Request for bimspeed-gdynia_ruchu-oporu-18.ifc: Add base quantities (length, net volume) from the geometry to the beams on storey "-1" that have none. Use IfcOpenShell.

First a look at what the model holds.

```python
import ifcopenshell
import ifcopenshell.util.element
import ifcopenshell.util.unit

model = ifcopenshell.open("bimspeed-gdynia_ruchu-oporu-18.ifc")
print(model.schema)
for unit_type in ("LENGTHUNIT", "AREAUNIT", "VOLUMEUNIT"):
    print(unit_type, ifcopenshell.util.unit.calculate_unit_scale(model, unit_type))
storey = next(s for s in model.by_type("IfcBuildingStorey") if s.Name == "-1")
beams = [e for e in ifcopenshell.util.element.get_decomposition(storey) if e.is_a("IfcBeam")]
for e in sorted(beams, key=lambda e: e.id()):
    print(e.id(), e.is_a(), e.Name, list(ifcopenshell.util.element.get_psets(e, qtos_only=True)), sep=" | ")
```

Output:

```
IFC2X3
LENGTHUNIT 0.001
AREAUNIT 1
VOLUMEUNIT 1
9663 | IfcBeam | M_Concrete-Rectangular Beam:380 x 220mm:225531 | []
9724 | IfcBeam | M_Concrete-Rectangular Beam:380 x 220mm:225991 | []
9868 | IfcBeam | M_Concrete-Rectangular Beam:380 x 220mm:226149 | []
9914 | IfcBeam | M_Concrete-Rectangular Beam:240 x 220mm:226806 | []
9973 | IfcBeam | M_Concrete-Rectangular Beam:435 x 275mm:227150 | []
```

```python
import ifcopenshell
import ifcopenshell.api.pset
import ifcopenshell.geom
import ifcopenshell.util.element
import ifcopenshell.util.shape
import ifcopenshell.util.unit

model = ifcopenshell.open("bimspeed-gdynia_ruchu-oporu-18.ifc")
unit_scale = ifcopenshell.util.unit.calculate_unit_scale(model)
volume_scale = ifcopenshell.util.unit.calculate_unit_scale(model, "VOLUMEUNIT")
settings = ifcopenshell.geom.settings()

storey = next(s for s in model.by_type("IfcBuildingStorey") if s.Name == "-1")
beams = [e for e in ifcopenshell.util.element.get_decomposition(storey) if e.is_a("IfcBeam")]

for e in sorted(beams, key=lambda e: e.id()):
    if ifcopenshell.util.element.get_psets(e, qtos_only=True, should_inherit=False):
        continue
    # Geometry comes back in metres, in the element's own axes.
    shape = ifcopenshell.geom.create_shape(settings, e)
    values = {
        "Length": ifcopenshell.util.shape.get_max_xyz(shape.geometry) / unit_scale,
        "NetVolume": ifcopenshell.util.shape.get_volume(shape.geometry) / volume_scale,
    }
    qto = ifcopenshell.api.pset.add_qto(model, product=e, name="BaseQuantities")
    ifcopenshell.api.pset.edit_qto(model, qto=qto, properties=values)
    print(e.id(), {k: round(v, 3) for k, v in values.items()})

model.write("bimspeed-gdynia_ruchu-oporu-18_updated.ifc")
```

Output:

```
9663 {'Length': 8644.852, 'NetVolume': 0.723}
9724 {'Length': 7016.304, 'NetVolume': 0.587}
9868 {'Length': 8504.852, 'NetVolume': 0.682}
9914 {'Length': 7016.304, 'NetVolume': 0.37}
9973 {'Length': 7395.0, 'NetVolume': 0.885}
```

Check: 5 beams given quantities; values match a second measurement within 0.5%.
